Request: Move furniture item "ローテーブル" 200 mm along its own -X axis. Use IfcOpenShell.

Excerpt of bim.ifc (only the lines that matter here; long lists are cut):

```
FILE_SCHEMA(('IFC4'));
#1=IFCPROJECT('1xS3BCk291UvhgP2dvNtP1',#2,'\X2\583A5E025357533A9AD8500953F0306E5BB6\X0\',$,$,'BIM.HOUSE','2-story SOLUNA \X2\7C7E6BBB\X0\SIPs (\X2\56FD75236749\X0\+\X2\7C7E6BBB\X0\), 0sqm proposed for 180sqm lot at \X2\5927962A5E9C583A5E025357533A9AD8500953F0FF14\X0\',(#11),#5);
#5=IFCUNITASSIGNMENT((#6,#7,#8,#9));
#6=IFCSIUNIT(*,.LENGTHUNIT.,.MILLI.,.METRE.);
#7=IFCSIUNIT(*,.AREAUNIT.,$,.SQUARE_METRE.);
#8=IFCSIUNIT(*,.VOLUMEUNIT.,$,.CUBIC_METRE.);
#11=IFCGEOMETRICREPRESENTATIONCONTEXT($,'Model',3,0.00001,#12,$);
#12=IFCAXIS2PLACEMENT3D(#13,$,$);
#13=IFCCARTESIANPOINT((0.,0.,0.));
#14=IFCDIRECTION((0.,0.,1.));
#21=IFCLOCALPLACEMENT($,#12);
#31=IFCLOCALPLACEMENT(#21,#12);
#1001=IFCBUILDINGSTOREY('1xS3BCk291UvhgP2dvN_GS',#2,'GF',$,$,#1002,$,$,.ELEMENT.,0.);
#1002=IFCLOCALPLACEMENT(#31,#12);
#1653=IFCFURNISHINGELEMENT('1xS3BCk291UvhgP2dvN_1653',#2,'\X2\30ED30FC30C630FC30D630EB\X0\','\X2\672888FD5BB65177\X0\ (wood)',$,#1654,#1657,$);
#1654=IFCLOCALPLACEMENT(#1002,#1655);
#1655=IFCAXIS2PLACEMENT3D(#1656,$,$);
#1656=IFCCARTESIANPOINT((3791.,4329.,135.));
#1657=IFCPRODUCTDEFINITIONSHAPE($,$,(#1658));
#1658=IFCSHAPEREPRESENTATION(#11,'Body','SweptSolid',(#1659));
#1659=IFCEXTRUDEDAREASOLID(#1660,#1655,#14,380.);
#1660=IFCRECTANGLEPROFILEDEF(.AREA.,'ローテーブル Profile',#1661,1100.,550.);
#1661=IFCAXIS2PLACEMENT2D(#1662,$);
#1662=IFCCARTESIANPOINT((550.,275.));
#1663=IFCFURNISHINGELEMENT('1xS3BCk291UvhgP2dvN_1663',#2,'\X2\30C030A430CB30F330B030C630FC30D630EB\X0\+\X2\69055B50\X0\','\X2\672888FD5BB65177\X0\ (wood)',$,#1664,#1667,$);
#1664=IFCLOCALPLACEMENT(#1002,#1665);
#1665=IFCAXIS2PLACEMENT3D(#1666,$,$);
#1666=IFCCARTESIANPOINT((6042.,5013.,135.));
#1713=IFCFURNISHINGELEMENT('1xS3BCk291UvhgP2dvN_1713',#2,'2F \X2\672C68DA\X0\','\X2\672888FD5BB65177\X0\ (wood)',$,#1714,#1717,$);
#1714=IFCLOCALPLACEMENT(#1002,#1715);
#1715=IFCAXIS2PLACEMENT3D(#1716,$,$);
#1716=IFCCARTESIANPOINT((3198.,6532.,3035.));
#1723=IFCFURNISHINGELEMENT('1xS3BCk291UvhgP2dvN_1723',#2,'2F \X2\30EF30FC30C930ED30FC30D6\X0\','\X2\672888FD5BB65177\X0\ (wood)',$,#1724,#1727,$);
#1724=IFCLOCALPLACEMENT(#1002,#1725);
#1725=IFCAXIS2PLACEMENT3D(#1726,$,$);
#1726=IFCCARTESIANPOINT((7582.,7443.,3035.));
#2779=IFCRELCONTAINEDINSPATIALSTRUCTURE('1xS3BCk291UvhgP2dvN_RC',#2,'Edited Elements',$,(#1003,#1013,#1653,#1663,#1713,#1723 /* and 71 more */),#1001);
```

```python
import ifcopenshell
import ifcopenshell.api.geometry
import ifcopenshell.util.placement

model = ifcopenshell.open("bim.ifc")

item = model.by_id(1653)
matrix = ifcopenshell.util.placement.get_local_placement(item.ObjectPlacement)
matrix[:3, 3] -= matrix[:3, 0] * 200.0
ifcopenshell.api.geometry.edit_object_placement(model, product=item, matrix=matrix, is_si=False)

print(ifcopenshell.util.placement.get_local_placement(item.ObjectPlacement).round(3) + 0.0)

model.write("bim_updated.ifc")
```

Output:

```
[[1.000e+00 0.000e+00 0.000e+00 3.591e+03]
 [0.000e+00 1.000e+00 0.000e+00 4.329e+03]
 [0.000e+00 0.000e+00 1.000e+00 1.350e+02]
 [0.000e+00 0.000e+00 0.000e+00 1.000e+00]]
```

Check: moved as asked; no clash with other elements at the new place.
